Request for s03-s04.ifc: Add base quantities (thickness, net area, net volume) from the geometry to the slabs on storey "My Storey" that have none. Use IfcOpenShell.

First a look at what the model holds.

```python
import ifcopenshell
import ifcopenshell.util.element
import ifcopenshell.util.unit

model = ifcopenshell.open("s03-s04.ifc")
print(model.schema)
for unit_type in ("LENGTHUNIT", "AREAUNIT", "VOLUMEUNIT"):
    print(unit_type, ifcopenshell.util.unit.calculate_unit_scale(model, unit_type))
storey = next(s for s in model.by_type("IfcBuildingStorey") if s.Name == "My Storey")
slabs = [e for e in ifcopenshell.util.element.get_decomposition(storey) if e.is_a("IfcSlab")]
for e in sorted(slabs, key=lambda e: e.id()):
    print(e.id(), e.is_a(), e.Name, list(ifcopenshell.util.element.get_psets(e, qtos_only=True)), sep=" | ")
```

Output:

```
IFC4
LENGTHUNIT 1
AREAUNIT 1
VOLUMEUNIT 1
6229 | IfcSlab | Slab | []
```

```python
import ifcopenshell
import ifcopenshell.api.pset
import ifcopenshell.geom
import ifcopenshell.util.element
import ifcopenshell.util.shape
import ifcopenshell.util.unit

model = ifcopenshell.open("s03-s04.ifc")
unit_scale = ifcopenshell.util.unit.calculate_unit_scale(model)
area_scale = ifcopenshell.util.unit.calculate_unit_scale(model, "AREAUNIT")
volume_scale = ifcopenshell.util.unit.calculate_unit_scale(model, "VOLUMEUNIT")
settings = ifcopenshell.geom.settings()

storey = next(s for s in model.by_type("IfcBuildingStorey") if s.Name == "My Storey")
slabs = [e for e in ifcopenshell.util.element.get_decomposition(storey) if e.is_a("IfcSlab")]

for e in sorted(slabs, key=lambda e: e.id()):
    if ifcopenshell.util.element.get_psets(e, qtos_only=True, should_inherit=False):
        continue
    # Geometry comes back in metres, in the element's own axes.
    shape = ifcopenshell.geom.create_shape(settings, e)
    values = {
        "Width": ifcopenshell.util.shape.get_z(shape.geometry) / unit_scale,
        "NetArea": ifcopenshell.util.shape.get_footprint_area(shape.geometry) / area_scale,
        "NetVolume": ifcopenshell.util.shape.get_volume(shape.geometry) / volume_scale,
    }
    qto = ifcopenshell.api.pset.add_qto(model, product=e, name="Qto_SlabBaseQuantities")
    ifcopenshell.api.pset.edit_qto(model, qto=qto, properties=values)
    print(e.id(), {k: round(v, 3) for k, v in values.items()})

model.write("s03-s04-out.ifc")
```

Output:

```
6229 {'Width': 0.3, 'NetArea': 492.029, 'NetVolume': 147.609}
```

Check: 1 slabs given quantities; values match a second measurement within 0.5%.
